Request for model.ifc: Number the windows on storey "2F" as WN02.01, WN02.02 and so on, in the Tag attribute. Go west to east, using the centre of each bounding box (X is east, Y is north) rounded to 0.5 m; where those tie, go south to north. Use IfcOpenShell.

First a look at what the model holds.

```python
import ifcopenshell
import ifcopenshell.util.element
import ifcopenshell.util.placement

model = ifcopenshell.open("model.ifc")
print(model.schema)
storey = next(s for s in model.by_type("IfcBuildingStorey") if s.Name == "2F")
windows = [e for e in ifcopenshell.util.element.get_decomposition(storey) if e.is_a("IfcWindow")]
for e in sorted(windows, key=lambda e: e.id()):
    origin = ifcopenshell.util.placement.get_local_placement(e.ObjectPlacement)[:3, 3]
    print(e.id(), e.Tag, e.Name, origin.round(2) + 0.0, sep=" | ")
```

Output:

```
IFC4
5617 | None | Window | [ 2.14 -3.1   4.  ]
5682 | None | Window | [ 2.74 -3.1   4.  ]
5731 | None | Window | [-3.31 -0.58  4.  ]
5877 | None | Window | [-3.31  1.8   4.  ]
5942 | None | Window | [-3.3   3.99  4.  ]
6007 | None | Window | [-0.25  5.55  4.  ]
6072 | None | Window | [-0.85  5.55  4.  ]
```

```python
import ifcopenshell
import ifcopenshell.geom
import ifcopenshell.util.element
import ifcopenshell.util.shape

model = ifcopenshell.open("model.ifc")
settings = ifcopenshell.geom.settings()
settings.set("use-world-coords", True)


def centre(element):
    shape = ifcopenshell.geom.create_shape(settings, element)
    return ifcopenshell.util.shape.get_bbox_centroid(shape.geometry)


storey = next(s for s in model.by_type("IfcBuildingStorey") if s.Name == "2F")
windows = [e for e in ifcopenshell.util.element.get_decomposition(storey) if e.is_a("IfcWindow")]

# Insertion points can sit at a corner or the storey origin, so sort by the geometry (in metres).
centres = {e: centre(e) for e in windows}
windows.sort(key=lambda e: (round(centres[e][0] / 0.5), centres[e][1]))

for i, e in enumerate(windows, start=1):
    number = f"WN02.{i:02d}"
    e.Tag = number
    print(e.id(), number)

model.write("model-out.ifc")
```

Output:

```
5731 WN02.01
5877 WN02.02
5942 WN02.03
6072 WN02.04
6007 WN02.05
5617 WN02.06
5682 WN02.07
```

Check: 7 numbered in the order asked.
